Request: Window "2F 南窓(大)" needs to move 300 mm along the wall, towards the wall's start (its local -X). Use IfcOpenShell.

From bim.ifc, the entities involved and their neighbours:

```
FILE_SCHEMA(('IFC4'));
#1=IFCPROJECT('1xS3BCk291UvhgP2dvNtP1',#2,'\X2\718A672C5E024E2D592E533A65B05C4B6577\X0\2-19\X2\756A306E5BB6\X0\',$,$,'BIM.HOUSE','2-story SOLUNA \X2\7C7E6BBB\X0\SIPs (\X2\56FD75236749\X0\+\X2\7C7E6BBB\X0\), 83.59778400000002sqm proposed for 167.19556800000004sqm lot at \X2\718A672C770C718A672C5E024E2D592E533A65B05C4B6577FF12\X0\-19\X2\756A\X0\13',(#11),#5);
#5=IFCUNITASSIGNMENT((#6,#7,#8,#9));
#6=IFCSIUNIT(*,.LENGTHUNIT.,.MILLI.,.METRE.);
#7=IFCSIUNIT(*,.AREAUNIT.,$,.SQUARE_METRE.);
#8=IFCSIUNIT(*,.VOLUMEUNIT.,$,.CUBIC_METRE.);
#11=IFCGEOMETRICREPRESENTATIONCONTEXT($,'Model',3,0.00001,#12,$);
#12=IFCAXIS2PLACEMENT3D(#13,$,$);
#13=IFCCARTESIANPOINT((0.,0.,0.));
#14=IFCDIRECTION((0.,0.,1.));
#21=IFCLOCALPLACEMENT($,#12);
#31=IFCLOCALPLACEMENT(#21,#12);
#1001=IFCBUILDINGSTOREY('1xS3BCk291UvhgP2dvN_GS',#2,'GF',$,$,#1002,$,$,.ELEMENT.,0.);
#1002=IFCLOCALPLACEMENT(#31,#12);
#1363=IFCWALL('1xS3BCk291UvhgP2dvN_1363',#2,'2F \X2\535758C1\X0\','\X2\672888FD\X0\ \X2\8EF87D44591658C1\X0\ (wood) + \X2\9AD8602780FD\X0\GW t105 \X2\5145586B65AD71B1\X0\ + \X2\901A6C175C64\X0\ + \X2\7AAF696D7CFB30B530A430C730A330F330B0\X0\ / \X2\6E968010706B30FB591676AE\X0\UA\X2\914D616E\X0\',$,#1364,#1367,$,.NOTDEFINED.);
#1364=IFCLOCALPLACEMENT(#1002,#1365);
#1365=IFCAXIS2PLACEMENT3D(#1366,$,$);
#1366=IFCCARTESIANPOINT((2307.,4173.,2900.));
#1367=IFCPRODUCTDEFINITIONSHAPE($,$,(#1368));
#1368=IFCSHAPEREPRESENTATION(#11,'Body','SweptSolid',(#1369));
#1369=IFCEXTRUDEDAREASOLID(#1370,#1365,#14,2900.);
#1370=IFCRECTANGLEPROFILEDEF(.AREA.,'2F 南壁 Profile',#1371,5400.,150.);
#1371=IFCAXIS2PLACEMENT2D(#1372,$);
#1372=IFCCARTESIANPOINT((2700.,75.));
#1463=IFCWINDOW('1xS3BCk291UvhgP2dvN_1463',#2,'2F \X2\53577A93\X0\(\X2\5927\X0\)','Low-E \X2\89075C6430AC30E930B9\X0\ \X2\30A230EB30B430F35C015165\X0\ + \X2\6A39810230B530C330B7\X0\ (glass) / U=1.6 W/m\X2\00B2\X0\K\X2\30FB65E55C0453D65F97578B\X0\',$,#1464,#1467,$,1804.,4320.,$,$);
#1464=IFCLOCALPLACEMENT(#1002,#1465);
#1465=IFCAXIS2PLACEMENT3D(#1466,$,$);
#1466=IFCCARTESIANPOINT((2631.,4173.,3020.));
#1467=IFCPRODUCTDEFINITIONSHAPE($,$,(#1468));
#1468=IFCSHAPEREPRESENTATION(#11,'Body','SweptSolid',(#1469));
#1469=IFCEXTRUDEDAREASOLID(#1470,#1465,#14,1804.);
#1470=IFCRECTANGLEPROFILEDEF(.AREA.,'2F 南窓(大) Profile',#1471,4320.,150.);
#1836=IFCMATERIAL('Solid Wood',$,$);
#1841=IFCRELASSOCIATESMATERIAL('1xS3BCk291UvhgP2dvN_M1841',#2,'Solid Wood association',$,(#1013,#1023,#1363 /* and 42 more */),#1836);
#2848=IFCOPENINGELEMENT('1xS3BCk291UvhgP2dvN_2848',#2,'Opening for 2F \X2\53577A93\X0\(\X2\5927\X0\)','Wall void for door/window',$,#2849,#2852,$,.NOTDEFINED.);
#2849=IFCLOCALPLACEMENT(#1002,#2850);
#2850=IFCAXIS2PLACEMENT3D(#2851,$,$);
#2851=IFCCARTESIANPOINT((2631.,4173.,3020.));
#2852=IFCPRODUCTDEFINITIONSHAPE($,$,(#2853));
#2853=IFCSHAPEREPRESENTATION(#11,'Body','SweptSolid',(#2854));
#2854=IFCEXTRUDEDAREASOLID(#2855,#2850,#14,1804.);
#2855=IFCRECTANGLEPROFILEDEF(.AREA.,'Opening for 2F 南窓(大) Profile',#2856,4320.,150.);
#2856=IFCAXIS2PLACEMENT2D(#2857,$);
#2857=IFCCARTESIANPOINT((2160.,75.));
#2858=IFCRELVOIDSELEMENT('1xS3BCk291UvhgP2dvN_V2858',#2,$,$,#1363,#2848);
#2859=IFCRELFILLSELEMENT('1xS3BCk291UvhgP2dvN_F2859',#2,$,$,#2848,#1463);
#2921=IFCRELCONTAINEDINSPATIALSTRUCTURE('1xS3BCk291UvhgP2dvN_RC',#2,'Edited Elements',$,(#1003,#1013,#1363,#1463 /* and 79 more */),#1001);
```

```python
import ifcopenshell
import ifcopenshell.api.geometry
import ifcopenshell.util.placement

model = ifcopenshell.open("bim.ifc")

window = model.by_guid("1xS3BCk291UvhgP2dvN_1463")
opening = window.FillsVoids[0].RelatingOpeningElement
wall = opening.VoidsElements[0].RelatingBuildingElement

wall_matrix = ifcopenshell.util.placement.get_local_placement(wall.ObjectPlacement)
shift = wall_matrix[:3, 0] * -300.0
before = ifcopenshell.util.placement.get_local_placement(window.ObjectPlacement)[:3, 3].copy()

# The window is not placed relative to its opening, so move both.
for product in (opening, window):
    matrix = ifcopenshell.util.placement.get_local_placement(product.ObjectPlacement)
    matrix[:3, 3] += shift
    ifcopenshell.api.geometry.edit_object_placement(model, product=product, matrix=matrix, is_si=False)

after = ifcopenshell.util.placement.get_local_placement(window.ObjectPlacement)[:3, 3]
print("window moved by", (after - before).round(3) + 0.0)

model.write("bim_rev.ifc")
```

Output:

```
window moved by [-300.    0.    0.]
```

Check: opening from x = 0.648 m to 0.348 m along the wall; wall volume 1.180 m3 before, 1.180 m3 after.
